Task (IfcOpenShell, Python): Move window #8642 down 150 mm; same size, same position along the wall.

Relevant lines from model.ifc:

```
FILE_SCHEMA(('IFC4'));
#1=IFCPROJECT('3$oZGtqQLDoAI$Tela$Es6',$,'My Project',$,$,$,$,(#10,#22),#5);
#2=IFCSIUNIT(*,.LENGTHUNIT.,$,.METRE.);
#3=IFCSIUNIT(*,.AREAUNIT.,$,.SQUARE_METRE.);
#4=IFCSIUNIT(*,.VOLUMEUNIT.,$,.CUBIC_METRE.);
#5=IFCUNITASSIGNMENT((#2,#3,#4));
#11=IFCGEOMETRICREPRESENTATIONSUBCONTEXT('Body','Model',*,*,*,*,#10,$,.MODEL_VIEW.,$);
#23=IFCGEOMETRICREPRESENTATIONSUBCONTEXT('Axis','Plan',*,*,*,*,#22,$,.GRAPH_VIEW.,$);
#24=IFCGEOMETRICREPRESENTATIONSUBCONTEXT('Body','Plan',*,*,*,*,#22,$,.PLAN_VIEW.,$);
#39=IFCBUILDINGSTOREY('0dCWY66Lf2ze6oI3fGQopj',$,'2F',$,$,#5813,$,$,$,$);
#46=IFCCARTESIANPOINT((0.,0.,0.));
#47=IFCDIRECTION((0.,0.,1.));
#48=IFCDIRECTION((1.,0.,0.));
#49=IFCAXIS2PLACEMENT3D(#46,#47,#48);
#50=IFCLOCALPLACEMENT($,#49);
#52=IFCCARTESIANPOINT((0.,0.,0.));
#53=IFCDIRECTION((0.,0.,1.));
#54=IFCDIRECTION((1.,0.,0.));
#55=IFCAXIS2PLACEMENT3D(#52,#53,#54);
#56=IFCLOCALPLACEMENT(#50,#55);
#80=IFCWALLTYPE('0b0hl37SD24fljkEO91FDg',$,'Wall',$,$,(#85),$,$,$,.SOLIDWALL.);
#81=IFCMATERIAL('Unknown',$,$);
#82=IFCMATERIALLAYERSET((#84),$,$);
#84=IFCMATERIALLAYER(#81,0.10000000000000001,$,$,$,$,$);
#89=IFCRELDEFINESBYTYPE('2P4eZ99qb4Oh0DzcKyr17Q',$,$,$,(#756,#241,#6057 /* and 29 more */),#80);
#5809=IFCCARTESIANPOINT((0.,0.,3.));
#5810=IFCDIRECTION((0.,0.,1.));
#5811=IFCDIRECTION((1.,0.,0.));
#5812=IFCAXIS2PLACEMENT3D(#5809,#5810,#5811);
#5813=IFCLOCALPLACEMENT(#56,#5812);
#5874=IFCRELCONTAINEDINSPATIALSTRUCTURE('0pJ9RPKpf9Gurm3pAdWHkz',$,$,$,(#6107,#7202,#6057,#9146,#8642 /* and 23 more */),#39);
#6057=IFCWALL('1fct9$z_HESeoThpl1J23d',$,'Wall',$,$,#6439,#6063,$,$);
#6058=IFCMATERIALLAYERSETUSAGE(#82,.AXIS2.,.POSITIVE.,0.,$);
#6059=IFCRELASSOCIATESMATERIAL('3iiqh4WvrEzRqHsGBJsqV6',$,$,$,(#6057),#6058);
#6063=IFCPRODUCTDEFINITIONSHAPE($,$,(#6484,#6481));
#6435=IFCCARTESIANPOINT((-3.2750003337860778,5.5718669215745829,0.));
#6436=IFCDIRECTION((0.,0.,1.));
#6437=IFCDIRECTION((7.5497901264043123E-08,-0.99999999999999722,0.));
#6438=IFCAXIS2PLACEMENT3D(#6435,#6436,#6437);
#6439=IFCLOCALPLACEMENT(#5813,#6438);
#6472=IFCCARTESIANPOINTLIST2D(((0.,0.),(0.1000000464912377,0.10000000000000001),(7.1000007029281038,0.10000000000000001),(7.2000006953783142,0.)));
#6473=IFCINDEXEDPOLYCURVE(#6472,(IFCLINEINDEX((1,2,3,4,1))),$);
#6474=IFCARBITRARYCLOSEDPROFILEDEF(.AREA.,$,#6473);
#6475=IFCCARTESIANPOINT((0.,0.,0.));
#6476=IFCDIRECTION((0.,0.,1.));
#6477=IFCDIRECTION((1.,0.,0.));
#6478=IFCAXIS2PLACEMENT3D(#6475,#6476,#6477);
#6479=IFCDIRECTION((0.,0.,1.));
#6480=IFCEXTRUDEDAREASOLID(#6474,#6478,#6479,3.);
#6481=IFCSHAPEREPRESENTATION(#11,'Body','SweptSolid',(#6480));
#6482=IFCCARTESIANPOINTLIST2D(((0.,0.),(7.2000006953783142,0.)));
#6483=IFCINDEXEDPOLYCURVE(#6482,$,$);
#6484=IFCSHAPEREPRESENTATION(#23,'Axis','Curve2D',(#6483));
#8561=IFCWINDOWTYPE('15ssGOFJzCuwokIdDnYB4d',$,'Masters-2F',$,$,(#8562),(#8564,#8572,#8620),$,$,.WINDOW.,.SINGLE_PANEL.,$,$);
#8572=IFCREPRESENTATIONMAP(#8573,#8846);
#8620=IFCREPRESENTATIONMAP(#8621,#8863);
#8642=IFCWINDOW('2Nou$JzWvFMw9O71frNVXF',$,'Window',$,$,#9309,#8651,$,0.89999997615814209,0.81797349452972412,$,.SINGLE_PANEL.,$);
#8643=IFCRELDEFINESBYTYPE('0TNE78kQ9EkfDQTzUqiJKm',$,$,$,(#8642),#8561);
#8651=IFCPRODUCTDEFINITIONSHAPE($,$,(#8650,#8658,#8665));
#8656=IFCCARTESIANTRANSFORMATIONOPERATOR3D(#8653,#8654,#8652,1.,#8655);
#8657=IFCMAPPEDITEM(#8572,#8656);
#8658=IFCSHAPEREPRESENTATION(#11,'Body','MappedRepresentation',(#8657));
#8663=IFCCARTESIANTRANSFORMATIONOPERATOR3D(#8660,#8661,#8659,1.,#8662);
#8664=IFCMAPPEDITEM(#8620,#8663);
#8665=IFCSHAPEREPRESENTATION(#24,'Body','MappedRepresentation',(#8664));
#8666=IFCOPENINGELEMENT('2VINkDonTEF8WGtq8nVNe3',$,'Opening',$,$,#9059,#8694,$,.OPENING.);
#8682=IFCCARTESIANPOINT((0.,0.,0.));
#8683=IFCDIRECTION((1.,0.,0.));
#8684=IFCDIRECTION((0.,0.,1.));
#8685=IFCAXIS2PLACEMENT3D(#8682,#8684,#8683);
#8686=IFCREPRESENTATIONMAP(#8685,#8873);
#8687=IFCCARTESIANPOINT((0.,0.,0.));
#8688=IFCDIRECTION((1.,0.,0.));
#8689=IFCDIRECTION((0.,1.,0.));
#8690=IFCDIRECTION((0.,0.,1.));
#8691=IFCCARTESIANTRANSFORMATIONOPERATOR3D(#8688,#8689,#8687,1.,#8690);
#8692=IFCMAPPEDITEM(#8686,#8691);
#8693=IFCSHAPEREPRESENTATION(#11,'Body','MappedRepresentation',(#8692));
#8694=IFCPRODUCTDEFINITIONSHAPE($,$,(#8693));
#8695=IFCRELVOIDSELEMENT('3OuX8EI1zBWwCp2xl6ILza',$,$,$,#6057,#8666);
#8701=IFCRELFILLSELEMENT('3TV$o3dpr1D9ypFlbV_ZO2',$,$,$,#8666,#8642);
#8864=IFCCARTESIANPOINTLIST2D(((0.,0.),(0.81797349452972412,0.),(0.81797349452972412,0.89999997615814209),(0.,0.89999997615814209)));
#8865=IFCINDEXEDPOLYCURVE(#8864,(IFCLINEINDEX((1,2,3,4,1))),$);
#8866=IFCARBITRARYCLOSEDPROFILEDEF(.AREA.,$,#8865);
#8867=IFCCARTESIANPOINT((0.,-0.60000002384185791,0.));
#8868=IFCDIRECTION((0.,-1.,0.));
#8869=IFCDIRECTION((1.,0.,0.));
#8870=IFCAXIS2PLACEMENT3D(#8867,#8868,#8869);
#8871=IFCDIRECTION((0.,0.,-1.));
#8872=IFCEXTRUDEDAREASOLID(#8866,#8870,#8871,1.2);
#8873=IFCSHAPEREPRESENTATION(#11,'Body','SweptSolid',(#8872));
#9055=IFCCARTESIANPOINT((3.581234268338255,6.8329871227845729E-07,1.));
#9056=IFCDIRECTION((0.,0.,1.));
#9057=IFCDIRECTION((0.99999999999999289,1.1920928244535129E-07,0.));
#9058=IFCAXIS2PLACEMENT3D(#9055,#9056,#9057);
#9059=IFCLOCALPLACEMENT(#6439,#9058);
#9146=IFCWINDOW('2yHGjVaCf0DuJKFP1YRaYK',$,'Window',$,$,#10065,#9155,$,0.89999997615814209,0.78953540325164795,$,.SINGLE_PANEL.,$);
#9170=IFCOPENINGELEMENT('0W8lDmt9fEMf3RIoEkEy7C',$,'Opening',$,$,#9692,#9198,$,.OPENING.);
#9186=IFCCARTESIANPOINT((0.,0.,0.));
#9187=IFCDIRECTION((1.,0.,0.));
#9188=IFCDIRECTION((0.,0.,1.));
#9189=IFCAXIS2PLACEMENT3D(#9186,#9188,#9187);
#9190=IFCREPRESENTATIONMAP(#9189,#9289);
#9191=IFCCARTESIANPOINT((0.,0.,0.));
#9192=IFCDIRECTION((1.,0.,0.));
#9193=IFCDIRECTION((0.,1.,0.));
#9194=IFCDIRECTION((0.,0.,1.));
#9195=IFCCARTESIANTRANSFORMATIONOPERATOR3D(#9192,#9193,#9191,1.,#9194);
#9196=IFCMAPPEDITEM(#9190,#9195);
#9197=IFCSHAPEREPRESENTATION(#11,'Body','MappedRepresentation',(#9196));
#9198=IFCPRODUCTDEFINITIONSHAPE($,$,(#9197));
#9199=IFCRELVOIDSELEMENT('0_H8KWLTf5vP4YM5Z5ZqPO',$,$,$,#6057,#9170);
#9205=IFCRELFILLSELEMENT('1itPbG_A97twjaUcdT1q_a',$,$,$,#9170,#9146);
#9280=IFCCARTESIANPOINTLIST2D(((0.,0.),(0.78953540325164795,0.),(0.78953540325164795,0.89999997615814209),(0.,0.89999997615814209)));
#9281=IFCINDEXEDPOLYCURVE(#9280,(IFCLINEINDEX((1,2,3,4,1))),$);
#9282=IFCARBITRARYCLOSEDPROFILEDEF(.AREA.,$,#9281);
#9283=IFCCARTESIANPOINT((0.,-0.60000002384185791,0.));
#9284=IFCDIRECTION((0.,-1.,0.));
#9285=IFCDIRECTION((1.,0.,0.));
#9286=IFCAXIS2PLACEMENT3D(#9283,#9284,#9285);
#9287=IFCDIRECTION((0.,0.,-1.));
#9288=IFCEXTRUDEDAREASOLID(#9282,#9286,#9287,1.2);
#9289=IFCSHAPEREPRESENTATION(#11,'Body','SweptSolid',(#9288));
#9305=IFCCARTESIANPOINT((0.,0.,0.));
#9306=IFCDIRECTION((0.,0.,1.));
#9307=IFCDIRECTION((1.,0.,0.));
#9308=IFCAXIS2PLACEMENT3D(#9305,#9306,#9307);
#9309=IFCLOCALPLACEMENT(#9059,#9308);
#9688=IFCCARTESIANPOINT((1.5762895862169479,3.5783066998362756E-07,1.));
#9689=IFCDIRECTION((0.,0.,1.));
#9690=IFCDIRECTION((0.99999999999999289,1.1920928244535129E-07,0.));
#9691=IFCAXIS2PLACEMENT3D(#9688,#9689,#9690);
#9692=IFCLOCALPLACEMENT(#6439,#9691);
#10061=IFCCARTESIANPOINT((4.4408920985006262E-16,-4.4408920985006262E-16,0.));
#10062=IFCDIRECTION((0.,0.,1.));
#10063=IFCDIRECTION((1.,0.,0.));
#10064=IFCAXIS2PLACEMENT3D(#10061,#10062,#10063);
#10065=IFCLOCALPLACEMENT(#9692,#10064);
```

```python
import numpy as np
import ifcopenshell
import ifcopenshell.api.geometry
import ifcopenshell.util.placement
import ifcopenshell.util.unit

model = ifcopenshell.open("model.ifc")
unit_scale = ifcopenshell.util.unit.calculate_unit_scale(model)

window = model.by_guid("2Nou$JzWvFMw9O71frNVXF")
opening = window.FillsVoids[0].RelatingOpeningElement
dz = -0.15 / unit_scale

shift = np.array([0.0, 0.0, dz])
# The window is placed relative to its opening, so it follows when the opening moves.
matrix = ifcopenshell.util.placement.get_local_placement(opening.ObjectPlacement)
matrix[:3, 3] += shift
ifcopenshell.api.geometry.edit_object_placement(
    model, product=opening, matrix=matrix, is_si=False, should_transform_children=True
)

print(f"moved by {dz * unit_scale:+.3f} m")

model.write("model_updated.ifc")
```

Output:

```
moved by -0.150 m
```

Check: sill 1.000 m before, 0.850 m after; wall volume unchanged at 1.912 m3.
